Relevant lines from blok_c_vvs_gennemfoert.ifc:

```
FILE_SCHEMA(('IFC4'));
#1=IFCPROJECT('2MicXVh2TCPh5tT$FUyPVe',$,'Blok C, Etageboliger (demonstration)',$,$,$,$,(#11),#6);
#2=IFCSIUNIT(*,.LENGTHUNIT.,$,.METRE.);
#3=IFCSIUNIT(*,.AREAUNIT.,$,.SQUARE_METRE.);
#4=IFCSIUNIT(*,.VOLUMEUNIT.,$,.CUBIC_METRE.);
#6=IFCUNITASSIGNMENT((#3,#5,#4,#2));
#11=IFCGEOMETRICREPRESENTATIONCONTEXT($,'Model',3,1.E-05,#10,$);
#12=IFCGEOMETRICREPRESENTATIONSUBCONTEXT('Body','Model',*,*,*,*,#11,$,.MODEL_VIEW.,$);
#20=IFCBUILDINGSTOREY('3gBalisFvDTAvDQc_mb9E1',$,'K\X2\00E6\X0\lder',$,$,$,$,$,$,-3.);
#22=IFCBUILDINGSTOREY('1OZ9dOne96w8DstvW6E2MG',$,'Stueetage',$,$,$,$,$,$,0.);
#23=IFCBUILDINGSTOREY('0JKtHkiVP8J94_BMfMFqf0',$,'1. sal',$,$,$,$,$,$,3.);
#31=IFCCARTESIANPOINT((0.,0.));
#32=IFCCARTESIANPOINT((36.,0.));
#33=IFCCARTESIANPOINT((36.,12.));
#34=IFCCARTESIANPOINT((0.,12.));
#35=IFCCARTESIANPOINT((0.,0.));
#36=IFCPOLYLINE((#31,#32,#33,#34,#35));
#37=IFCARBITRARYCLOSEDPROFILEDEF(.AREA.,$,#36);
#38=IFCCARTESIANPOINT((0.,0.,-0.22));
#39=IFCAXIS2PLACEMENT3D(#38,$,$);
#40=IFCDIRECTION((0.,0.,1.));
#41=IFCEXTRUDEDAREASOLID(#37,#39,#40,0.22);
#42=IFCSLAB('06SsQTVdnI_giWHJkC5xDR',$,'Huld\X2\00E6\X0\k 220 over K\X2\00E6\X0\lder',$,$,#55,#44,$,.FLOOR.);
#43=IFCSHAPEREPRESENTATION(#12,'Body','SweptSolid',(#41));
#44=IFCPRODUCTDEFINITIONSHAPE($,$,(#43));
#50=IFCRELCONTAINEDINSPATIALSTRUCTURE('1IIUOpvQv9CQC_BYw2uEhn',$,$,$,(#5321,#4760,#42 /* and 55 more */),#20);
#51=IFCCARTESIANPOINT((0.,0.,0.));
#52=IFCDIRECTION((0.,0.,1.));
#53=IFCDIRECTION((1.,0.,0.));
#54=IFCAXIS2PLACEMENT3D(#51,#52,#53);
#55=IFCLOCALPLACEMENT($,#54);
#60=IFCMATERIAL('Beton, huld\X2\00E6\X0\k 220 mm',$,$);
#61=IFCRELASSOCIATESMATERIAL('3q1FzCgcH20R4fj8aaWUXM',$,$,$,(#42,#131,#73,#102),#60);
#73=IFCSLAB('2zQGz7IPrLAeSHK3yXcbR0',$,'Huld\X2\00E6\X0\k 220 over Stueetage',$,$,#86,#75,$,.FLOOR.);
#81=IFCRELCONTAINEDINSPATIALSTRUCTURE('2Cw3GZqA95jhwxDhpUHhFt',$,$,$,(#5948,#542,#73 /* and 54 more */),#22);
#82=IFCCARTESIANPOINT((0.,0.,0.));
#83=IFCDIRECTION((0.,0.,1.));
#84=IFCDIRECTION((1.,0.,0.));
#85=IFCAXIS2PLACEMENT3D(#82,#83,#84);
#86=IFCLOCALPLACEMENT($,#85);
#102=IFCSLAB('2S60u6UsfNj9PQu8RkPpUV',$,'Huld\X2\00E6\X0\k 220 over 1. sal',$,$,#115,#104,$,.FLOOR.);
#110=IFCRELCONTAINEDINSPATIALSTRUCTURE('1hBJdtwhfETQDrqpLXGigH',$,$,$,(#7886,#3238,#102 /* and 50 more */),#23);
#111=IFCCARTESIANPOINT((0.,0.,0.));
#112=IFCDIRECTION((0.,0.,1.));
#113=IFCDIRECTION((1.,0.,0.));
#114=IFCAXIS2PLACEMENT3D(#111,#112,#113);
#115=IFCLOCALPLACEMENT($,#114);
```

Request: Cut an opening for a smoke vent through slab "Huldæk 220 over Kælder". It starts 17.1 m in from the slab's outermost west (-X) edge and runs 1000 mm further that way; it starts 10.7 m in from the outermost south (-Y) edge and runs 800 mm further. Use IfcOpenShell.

```python
import numpy as np
import ifcopenshell
import ifcopenshell.api.feature
import ifcopenshell.api.geometry
import ifcopenshell.api.root
import ifcopenshell.geom
import ifcopenshell.util.placement
import ifcopenshell.util.representation
import ifcopenshell.util.shape
import ifcopenshell.util.unit

model = ifcopenshell.open("blok_c_vvs_gennemfoert.ifc")
unit_scale = ifcopenshell.util.unit.calculate_unit_scale(model)
settings = ifcopenshell.geom.settings()


def volume(element):
    """Net volume in cubic metres, openings subtracted."""
    shape = ifcopenshell.geom.create_shape(settings, element)
    return ifcopenshell.util.shape.get_volume(shape.geometry)


slab = model.by_id(42)
before = volume(slab)

# Extent in the slab's own axes, in metres. The edges named are its -X and -Y sides.
slab_shape = ifcopenshell.geom.create_shape(settings, slab)
vertices = ifcopenshell.util.shape.get_vertices(slab_shape.geometry)
x_min, y_min, bottom = vertices.min(axis=0)
top = vertices[:, 2].max()

opening = ifcopenshell.api.root.create_entity(model, ifc_class="IfcOpeningElement", name="Smoke vent opening", predefined_type="OPENING")
context = ifcopenshell.util.representation.get_context(model, "Model", "Body", "MODEL_VIEW")
width, depth = 1, 0.8
outline = [(0.0, 0.0), (width, 0.0), (width, depth), (0.0, depth), (0.0, 0.0)]
# Overshoot both faces by 50 mm so the cut is clean.
shape = ifcopenshell.api.geometry.add_slab_representation(
    model, context=context, depth=top - bottom + 0.1, polyline=outline
)
ifcopenshell.api.geometry.assign_representation(model, product=opening, representation=shape)

matrix = ifcopenshell.util.placement.get_local_placement(slab.ObjectPlacement)
matrix[:, 3] = matrix @ np.append(np.array([x_min + 17.1, y_min + 10.7, bottom - 0.05]) / unit_scale, 1.0)
ifcopenshell.api.geometry.edit_object_placement(model, product=opening, matrix=matrix, is_si=False)
ifcopenshell.api.feature.add_feature(model, feature=opening, element=slab)

after = volume(slab)

print(f"slab volume {before:.3f} -> {after:.3f} m3")

model.write("blok_c_vvs_gennemfoert_updated.ifc")
```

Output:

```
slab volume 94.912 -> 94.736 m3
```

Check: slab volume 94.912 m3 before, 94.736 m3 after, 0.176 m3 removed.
